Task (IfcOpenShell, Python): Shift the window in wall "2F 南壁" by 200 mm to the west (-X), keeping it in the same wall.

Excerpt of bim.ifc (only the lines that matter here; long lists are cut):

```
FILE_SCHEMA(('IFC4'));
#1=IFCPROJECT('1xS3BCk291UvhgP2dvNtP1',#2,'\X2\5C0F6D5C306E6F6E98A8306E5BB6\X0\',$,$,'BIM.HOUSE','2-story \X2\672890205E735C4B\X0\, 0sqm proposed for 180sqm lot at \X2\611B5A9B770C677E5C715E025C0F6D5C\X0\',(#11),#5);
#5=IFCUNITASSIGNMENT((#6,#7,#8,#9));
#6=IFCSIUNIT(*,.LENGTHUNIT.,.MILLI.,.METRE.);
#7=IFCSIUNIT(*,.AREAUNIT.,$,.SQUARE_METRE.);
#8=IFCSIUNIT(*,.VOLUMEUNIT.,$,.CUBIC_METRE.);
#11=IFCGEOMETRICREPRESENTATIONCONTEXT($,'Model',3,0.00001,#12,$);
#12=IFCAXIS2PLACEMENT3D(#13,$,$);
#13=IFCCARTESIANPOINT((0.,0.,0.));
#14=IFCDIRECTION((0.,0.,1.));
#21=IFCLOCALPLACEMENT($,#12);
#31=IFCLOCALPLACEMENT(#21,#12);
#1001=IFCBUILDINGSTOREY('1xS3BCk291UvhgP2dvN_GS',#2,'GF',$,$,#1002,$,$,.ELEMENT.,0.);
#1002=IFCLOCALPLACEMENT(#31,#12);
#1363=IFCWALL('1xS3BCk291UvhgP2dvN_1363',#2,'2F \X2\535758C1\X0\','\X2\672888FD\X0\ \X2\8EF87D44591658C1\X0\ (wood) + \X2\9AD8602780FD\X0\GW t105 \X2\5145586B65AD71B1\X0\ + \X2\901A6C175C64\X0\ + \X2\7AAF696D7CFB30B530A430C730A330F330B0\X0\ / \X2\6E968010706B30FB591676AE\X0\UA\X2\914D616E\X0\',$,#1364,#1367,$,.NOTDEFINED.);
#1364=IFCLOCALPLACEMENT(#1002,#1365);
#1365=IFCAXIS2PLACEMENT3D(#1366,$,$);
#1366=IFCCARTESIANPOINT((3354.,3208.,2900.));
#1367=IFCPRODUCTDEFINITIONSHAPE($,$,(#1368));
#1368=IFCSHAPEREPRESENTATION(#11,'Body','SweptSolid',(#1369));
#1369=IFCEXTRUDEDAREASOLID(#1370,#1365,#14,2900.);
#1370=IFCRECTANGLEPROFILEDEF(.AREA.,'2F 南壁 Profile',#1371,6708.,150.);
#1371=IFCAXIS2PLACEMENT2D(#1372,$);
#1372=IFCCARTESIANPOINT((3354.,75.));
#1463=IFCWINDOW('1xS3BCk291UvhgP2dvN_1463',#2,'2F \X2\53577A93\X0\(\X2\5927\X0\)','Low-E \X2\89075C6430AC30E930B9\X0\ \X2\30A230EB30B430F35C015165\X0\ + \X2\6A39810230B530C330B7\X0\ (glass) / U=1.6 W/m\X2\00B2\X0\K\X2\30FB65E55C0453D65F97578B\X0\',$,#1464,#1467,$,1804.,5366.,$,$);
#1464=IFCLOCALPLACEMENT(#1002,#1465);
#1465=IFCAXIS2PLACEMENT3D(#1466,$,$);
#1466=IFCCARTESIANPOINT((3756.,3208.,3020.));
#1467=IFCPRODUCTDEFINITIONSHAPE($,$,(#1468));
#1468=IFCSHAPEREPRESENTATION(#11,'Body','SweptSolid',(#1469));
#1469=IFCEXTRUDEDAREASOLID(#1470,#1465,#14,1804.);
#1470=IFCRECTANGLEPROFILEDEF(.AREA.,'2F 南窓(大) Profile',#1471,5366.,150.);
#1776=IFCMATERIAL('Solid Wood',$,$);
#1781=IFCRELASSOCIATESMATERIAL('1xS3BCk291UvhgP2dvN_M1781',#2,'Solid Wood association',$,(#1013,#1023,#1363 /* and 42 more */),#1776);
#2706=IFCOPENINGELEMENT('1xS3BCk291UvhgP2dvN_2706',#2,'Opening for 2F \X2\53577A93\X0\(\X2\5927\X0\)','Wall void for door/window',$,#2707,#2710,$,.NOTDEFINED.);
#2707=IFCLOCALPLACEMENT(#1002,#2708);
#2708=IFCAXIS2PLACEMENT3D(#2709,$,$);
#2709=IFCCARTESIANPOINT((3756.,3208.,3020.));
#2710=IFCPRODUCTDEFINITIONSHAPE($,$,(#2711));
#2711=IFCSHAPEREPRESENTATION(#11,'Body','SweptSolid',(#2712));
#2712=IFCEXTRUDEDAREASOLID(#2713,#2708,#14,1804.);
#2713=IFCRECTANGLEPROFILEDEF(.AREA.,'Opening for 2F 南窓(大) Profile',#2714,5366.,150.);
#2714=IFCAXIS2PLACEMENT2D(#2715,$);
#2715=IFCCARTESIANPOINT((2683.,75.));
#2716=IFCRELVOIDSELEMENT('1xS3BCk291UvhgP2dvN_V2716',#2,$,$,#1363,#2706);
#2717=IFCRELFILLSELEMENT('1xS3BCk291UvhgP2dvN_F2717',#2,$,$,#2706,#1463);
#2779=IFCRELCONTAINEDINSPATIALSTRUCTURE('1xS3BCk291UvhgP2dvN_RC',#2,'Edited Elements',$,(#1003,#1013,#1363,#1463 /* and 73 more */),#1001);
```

```python
import ifcopenshell
import ifcopenshell.api.geometry
import ifcopenshell.util.placement
import ifcopenshell.util.unit

model = ifcopenshell.open("bim.ifc")
unit_scale = ifcopenshell.util.unit.calculate_unit_scale(model)

window = model.by_guid("1xS3BCk291UvhgP2dvN_1463")
opening = window.FillsVoids[0].RelatingOpeningElement
wall = opening.VoidsElements[0].RelatingBuildingElement

wall_matrix = ifcopenshell.util.placement.get_local_placement(wall.ObjectPlacement)
shift = wall_matrix[:3, 0] * -0.2 / unit_scale
before = ifcopenshell.util.placement.get_local_placement(window.ObjectPlacement)[:3, 3].copy()

# The window is not placed relative to its opening, so move both.
for product in (opening, window):
    matrix = ifcopenshell.util.placement.get_local_placement(product.ObjectPlacement)
    matrix[:3, 3] += shift
    ifcopenshell.api.geometry.edit_object_placement(model, product=product, matrix=matrix, is_si=False)

after = ifcopenshell.util.placement.get_local_placement(window.ObjectPlacement)[:3, 3]
print("window moved by", (after - before).round(3) + 0.0)

model.write("bim-out.ifc")
```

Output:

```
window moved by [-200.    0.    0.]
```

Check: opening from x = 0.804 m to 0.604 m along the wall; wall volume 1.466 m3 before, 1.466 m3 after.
